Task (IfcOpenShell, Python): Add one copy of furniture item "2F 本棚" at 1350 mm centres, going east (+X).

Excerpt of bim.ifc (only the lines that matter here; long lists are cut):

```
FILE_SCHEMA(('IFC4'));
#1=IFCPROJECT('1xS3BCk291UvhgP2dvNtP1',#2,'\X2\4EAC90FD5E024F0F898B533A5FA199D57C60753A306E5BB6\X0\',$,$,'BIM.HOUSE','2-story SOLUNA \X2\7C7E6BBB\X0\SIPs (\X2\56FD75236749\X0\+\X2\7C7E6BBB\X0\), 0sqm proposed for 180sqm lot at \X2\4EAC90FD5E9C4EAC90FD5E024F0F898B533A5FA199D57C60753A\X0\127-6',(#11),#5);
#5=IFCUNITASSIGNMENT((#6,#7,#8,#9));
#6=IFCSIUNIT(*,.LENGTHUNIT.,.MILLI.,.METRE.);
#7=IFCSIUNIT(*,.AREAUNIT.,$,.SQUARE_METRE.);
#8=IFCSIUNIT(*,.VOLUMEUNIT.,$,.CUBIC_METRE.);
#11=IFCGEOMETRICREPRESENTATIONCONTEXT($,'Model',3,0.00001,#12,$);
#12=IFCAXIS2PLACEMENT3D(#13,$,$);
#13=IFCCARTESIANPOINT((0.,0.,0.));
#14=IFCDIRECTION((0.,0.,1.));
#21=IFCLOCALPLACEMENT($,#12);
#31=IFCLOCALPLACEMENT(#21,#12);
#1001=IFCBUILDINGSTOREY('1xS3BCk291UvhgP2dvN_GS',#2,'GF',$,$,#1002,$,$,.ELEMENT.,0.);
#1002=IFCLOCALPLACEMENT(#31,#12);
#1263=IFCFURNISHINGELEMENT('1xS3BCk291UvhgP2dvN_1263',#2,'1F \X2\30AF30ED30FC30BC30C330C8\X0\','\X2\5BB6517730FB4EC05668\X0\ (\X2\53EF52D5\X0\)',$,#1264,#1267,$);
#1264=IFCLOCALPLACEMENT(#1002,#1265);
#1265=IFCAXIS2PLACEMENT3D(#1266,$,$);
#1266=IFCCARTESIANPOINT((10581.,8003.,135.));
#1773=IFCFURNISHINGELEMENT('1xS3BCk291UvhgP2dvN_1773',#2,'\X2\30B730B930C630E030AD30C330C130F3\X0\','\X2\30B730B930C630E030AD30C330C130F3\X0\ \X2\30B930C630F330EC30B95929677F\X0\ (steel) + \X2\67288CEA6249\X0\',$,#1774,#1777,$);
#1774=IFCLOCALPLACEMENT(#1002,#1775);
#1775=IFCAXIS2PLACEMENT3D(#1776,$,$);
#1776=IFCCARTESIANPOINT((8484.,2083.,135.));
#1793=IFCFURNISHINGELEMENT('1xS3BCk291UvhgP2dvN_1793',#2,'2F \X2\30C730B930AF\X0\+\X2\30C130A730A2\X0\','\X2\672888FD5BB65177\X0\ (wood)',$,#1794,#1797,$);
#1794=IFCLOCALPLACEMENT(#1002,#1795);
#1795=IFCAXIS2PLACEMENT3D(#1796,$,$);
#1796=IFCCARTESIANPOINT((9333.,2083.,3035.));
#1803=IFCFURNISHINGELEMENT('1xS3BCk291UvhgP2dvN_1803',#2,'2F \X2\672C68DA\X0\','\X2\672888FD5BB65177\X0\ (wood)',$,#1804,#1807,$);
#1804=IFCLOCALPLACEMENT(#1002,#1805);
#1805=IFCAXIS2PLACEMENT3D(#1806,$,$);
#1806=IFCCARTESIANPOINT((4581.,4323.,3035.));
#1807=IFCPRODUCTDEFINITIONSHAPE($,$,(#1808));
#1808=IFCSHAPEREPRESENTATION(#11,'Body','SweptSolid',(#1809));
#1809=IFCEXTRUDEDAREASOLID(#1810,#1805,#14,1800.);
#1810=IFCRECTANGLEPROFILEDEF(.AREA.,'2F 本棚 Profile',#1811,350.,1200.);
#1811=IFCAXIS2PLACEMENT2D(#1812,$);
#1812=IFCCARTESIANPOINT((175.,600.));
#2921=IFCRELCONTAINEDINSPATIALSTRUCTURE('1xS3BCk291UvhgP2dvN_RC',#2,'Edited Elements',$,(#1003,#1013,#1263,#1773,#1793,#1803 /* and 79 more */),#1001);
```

```python
import numpy as np
import ifcopenshell
import ifcopenshell.api.geometry
import ifcopenshell.api.root
import ifcopenshell.util.element
import ifcopenshell.util.placement

model = ifcopenshell.open("bim.ifc")


def reuse_history(source, copy):
    """copy_class also copies each property set's owner history, people and application; keep the originals."""
    for rel in copy.IsDefinedBy:
        if rel.is_a("IfcRelDefinesByProperties") and (history := rel.RelatingPropertyDefinition.OwnerHistory):
            rel.RelatingPropertyDefinition.OwnerHistory = source.OwnerHistory
            ifcopenshell.util.element.remove_deep2(model, history)


source = model.by_id(1803)
base = ifcopenshell.util.placement.get_local_placement(source.ObjectPlacement)
step = np.array([1.0, 0.0, 0.0]) * 1350.0

for i in range(1, 2):
    copy = ifcopenshell.api.root.copy_class(model, product=source)
    copy.Representation = ifcopenshell.util.element.copy_deep(
        model, source.Representation, exclude=["IfcGeometricRepresentationContext", "IfcRepresentationMap"]
    )
    reuse_history(source, copy)
    matrix = base.copy()
    matrix[:3, 3] += i * step
    print("added at", matrix[:3, 3].round(3) + 0.0)
    ifcopenshell.api.geometry.edit_object_placement(model, product=copy, matrix=matrix, is_si=False)

model.write("bim_v2.ifc")
```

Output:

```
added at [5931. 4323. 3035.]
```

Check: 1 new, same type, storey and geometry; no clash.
